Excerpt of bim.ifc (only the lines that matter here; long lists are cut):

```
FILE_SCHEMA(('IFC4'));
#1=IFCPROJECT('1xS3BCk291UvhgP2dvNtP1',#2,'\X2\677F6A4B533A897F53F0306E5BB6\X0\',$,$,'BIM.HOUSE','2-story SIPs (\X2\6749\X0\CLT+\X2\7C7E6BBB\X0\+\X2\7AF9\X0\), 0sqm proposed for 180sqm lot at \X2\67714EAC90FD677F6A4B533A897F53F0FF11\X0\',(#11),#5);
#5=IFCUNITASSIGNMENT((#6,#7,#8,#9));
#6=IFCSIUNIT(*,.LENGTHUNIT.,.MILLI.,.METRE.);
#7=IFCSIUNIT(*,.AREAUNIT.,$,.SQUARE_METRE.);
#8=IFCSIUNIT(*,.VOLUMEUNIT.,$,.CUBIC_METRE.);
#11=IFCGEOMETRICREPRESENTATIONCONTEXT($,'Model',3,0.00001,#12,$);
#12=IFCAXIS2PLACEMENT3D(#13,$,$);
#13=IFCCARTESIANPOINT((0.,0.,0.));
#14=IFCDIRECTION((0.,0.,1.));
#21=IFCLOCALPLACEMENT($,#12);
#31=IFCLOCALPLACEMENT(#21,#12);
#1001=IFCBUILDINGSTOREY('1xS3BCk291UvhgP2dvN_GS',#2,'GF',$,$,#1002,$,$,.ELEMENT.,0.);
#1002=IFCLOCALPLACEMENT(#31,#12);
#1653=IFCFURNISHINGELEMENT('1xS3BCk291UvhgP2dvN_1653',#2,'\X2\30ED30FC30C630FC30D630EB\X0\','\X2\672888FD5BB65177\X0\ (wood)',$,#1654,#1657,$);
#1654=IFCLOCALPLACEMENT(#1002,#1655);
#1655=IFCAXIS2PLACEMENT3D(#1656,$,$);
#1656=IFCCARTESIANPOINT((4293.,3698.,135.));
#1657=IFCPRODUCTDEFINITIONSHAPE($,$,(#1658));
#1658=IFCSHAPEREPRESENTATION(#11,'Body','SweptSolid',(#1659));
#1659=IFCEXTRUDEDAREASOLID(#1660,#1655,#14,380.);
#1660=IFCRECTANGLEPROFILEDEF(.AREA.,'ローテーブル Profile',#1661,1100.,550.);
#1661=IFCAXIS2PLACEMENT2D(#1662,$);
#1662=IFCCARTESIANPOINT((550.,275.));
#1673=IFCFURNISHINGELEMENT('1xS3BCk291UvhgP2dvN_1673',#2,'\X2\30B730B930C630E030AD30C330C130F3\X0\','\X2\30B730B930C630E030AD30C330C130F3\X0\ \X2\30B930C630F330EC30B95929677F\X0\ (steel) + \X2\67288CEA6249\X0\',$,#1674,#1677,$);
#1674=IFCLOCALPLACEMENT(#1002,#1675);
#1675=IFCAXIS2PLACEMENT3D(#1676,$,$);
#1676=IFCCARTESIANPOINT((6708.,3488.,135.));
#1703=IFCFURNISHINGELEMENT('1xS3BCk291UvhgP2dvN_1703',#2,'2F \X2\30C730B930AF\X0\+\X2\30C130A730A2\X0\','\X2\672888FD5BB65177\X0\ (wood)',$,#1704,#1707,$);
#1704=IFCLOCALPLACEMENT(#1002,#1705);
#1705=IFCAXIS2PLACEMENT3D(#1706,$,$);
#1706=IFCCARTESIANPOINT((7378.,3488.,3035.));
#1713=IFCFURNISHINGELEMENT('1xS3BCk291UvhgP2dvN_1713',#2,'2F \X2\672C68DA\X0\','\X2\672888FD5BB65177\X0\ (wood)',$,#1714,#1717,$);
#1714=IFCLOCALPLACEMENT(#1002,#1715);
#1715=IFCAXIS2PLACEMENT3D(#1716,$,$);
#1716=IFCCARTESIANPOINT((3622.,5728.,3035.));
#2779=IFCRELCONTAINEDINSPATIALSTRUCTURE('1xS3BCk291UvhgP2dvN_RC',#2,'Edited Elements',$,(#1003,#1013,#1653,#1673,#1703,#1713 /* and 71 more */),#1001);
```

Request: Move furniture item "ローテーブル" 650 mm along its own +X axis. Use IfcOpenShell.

```python
import ifcopenshell
import ifcopenshell.api.geometry
import ifcopenshell.util.placement

model = ifcopenshell.open("bim.ifc")

item = model.by_guid("1xS3BCk291UvhgP2dvN_1653")
matrix = ifcopenshell.util.placement.get_local_placement(item.ObjectPlacement)
matrix[:3, 3] += matrix[:3, 0] * 650.0
ifcopenshell.api.geometry.edit_object_placement(model, product=item, matrix=matrix, is_si=False)

print(ifcopenshell.util.placement.get_local_placement(item.ObjectPlacement).round(3) + 0.0)

model.write("bim-out.ifc")
```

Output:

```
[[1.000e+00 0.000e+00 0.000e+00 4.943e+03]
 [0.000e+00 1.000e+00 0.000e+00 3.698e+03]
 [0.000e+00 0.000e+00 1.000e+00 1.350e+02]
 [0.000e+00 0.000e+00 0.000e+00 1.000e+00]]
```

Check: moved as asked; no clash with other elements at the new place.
